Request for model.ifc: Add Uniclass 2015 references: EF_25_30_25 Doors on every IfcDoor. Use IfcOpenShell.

First a look at what the model holds.

```python
import ifcopenshell

model = ifcopenshell.open("model.ifc")
print(model.schema)
print("classifications:", [c.Name for c in model.by_type("IfcClassification")])
for ifc_class in ("IfcDoor", "IfcRoof", "IfcStair", "IfcWall", "IfcWindow"):
    print(ifc_class, len(model.by_type(ifc_class)))
```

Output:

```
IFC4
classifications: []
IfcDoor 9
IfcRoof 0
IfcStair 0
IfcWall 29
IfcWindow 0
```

```python
import ifcopenshell
import ifcopenshell.api.classification

model = ifcopenshell.open("model.ifc")

system = ifcopenshell.api.classification.add_classification(model, classification="Uniclass 2015")

codes = {
    "IfcDoor": ("EF_25_30_25", "Doors"),
}
for ifc_class, (code, name) in codes.items():
    products = model.by_type(ifc_class)
    ifcopenshell.api.classification.add_reference(
        model, products=products, classification=system, identification=code, name=name
    )
    print(code, len(products))

model.write("model_v2.ifc")
```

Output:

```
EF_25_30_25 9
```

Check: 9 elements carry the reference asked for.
